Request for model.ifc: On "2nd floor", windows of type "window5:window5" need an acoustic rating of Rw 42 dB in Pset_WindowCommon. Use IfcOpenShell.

First a look at what the model holds.

```python
import ifcopenshell
import ifcopenshell.util.element

model = ifcopenshell.open("model.ifc")
print(model.schema)
storey = next(s for s in model.by_type("IfcBuildingStorey") if s.Name == "2nd floor")
windows = [e for e in ifcopenshell.util.element.get_decomposition(storey) if e.is_a("IfcWindow")]
seen = {}
for e in windows:
    element_type = ifcopenshell.util.element.get_type(e)
    key = (element_type.Name if element_type != e and element_type else None, ifcopenshell.util.element.get_pset(e, "Pset_WindowCommon", "AcousticRating"))
    seen[key] = seen.get(key, 0) + 1
for (name, value), count in sorted(seen.items(), key=str):
    print(count, "x", name, "|", value)
```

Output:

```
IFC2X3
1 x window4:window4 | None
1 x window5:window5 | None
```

```python
import ifcopenshell
import ifcopenshell.api.pset
import ifcopenshell.util.element

model = ifcopenshell.open("model.ifc")

storey = next(s for s in model.by_type("IfcBuildingStorey") if s.Name == "2nd floor")
windows = [e for e in ifcopenshell.util.element.get_decomposition(storey) if e.is_a("IfcWindow")]

count = 0
for e in windows:
    element_type = ifcopenshell.util.element.get_type(e)
    if element_type in (None, e) or element_type.Name != "window5:window5":
        continue
    # add_pset returns the element's existing set when there is one.
    pset = ifcopenshell.api.pset.add_pset(model, product=e, name="Pset_WindowCommon")
    ifcopenshell.api.pset.edit_pset(model, pset=pset, properties={"AcousticRating": "Rw 42 dB"})
    count += 1

print(count, "windows updated")

model.write("model_v2.ifc")
```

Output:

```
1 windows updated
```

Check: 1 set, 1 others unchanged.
